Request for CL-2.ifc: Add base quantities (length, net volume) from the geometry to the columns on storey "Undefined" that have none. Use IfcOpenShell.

First a look at what the model holds.

```python
import ifcopenshell
import ifcopenshell.util.element
import ifcopenshell.util.unit

model = ifcopenshell.open("CL-2.ifc")
print(model.schema)
for unit_type in ("LENGTHUNIT", "AREAUNIT", "VOLUMEUNIT"):
    print(unit_type, ifcopenshell.util.unit.calculate_unit_scale(model, unit_type))
storey = next(s for s in model.by_type("IfcBuildingStorey") if s.Name == "Undefined")
columns = [e for e in ifcopenshell.util.element.get_decomposition(storey) if e.is_a("IfcColumn")]
for e in sorted(columns, key=lambda e: e.id()):
    print(e.id(), e.is_a(), e.Name, list(ifcopenshell.util.element.get_psets(e, qtos_only=True)), sep=" | ")
```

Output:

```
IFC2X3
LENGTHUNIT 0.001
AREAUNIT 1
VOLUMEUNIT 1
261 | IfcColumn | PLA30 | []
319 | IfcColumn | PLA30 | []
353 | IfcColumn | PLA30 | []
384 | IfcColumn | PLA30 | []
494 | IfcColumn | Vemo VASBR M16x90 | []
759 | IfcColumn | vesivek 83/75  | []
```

```python
import ifcopenshell
import ifcopenshell.api.pset
import ifcopenshell.geom
import ifcopenshell.util.element
import ifcopenshell.util.shape
import ifcopenshell.util.unit

model = ifcopenshell.open("CL-2.ifc")
unit_scale = ifcopenshell.util.unit.calculate_unit_scale(model)
volume_scale = ifcopenshell.util.unit.calculate_unit_scale(model, "VOLUMEUNIT")
settings = ifcopenshell.geom.settings()

storey = next(s for s in model.by_type("IfcBuildingStorey") if s.Name == "Undefined")
columns = [e for e in ifcopenshell.util.element.get_decomposition(storey) if e.is_a("IfcColumn")]

for e in sorted(columns, key=lambda e: e.id()):
    if ifcopenshell.util.element.get_psets(e, qtos_only=True, should_inherit=False):
        continue
    # Geometry comes back in metres, in the element's own axes.
    shape = ifcopenshell.geom.create_shape(settings, e)
    values = {
        "Length": ifcopenshell.util.shape.get_z(shape.geometry) / unit_scale,
        "NetVolume": ifcopenshell.util.shape.get_volume(shape.geometry) / volume_scale,
    }
    qto = ifcopenshell.api.pset.add_qto(model, product=e, name="BaseQuantities")
    ifcopenshell.api.pset.edit_qto(model, qto=qto, properties=values)
    print(e.id(), {k: round(v, 3) for k, v in values.items()})

model.write("CL-2_edited.ifc")
```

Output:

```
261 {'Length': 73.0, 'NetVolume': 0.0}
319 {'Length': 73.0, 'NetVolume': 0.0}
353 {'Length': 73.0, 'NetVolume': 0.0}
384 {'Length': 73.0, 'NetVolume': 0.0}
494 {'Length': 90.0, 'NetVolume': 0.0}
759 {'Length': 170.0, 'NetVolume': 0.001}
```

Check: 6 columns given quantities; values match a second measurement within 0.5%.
